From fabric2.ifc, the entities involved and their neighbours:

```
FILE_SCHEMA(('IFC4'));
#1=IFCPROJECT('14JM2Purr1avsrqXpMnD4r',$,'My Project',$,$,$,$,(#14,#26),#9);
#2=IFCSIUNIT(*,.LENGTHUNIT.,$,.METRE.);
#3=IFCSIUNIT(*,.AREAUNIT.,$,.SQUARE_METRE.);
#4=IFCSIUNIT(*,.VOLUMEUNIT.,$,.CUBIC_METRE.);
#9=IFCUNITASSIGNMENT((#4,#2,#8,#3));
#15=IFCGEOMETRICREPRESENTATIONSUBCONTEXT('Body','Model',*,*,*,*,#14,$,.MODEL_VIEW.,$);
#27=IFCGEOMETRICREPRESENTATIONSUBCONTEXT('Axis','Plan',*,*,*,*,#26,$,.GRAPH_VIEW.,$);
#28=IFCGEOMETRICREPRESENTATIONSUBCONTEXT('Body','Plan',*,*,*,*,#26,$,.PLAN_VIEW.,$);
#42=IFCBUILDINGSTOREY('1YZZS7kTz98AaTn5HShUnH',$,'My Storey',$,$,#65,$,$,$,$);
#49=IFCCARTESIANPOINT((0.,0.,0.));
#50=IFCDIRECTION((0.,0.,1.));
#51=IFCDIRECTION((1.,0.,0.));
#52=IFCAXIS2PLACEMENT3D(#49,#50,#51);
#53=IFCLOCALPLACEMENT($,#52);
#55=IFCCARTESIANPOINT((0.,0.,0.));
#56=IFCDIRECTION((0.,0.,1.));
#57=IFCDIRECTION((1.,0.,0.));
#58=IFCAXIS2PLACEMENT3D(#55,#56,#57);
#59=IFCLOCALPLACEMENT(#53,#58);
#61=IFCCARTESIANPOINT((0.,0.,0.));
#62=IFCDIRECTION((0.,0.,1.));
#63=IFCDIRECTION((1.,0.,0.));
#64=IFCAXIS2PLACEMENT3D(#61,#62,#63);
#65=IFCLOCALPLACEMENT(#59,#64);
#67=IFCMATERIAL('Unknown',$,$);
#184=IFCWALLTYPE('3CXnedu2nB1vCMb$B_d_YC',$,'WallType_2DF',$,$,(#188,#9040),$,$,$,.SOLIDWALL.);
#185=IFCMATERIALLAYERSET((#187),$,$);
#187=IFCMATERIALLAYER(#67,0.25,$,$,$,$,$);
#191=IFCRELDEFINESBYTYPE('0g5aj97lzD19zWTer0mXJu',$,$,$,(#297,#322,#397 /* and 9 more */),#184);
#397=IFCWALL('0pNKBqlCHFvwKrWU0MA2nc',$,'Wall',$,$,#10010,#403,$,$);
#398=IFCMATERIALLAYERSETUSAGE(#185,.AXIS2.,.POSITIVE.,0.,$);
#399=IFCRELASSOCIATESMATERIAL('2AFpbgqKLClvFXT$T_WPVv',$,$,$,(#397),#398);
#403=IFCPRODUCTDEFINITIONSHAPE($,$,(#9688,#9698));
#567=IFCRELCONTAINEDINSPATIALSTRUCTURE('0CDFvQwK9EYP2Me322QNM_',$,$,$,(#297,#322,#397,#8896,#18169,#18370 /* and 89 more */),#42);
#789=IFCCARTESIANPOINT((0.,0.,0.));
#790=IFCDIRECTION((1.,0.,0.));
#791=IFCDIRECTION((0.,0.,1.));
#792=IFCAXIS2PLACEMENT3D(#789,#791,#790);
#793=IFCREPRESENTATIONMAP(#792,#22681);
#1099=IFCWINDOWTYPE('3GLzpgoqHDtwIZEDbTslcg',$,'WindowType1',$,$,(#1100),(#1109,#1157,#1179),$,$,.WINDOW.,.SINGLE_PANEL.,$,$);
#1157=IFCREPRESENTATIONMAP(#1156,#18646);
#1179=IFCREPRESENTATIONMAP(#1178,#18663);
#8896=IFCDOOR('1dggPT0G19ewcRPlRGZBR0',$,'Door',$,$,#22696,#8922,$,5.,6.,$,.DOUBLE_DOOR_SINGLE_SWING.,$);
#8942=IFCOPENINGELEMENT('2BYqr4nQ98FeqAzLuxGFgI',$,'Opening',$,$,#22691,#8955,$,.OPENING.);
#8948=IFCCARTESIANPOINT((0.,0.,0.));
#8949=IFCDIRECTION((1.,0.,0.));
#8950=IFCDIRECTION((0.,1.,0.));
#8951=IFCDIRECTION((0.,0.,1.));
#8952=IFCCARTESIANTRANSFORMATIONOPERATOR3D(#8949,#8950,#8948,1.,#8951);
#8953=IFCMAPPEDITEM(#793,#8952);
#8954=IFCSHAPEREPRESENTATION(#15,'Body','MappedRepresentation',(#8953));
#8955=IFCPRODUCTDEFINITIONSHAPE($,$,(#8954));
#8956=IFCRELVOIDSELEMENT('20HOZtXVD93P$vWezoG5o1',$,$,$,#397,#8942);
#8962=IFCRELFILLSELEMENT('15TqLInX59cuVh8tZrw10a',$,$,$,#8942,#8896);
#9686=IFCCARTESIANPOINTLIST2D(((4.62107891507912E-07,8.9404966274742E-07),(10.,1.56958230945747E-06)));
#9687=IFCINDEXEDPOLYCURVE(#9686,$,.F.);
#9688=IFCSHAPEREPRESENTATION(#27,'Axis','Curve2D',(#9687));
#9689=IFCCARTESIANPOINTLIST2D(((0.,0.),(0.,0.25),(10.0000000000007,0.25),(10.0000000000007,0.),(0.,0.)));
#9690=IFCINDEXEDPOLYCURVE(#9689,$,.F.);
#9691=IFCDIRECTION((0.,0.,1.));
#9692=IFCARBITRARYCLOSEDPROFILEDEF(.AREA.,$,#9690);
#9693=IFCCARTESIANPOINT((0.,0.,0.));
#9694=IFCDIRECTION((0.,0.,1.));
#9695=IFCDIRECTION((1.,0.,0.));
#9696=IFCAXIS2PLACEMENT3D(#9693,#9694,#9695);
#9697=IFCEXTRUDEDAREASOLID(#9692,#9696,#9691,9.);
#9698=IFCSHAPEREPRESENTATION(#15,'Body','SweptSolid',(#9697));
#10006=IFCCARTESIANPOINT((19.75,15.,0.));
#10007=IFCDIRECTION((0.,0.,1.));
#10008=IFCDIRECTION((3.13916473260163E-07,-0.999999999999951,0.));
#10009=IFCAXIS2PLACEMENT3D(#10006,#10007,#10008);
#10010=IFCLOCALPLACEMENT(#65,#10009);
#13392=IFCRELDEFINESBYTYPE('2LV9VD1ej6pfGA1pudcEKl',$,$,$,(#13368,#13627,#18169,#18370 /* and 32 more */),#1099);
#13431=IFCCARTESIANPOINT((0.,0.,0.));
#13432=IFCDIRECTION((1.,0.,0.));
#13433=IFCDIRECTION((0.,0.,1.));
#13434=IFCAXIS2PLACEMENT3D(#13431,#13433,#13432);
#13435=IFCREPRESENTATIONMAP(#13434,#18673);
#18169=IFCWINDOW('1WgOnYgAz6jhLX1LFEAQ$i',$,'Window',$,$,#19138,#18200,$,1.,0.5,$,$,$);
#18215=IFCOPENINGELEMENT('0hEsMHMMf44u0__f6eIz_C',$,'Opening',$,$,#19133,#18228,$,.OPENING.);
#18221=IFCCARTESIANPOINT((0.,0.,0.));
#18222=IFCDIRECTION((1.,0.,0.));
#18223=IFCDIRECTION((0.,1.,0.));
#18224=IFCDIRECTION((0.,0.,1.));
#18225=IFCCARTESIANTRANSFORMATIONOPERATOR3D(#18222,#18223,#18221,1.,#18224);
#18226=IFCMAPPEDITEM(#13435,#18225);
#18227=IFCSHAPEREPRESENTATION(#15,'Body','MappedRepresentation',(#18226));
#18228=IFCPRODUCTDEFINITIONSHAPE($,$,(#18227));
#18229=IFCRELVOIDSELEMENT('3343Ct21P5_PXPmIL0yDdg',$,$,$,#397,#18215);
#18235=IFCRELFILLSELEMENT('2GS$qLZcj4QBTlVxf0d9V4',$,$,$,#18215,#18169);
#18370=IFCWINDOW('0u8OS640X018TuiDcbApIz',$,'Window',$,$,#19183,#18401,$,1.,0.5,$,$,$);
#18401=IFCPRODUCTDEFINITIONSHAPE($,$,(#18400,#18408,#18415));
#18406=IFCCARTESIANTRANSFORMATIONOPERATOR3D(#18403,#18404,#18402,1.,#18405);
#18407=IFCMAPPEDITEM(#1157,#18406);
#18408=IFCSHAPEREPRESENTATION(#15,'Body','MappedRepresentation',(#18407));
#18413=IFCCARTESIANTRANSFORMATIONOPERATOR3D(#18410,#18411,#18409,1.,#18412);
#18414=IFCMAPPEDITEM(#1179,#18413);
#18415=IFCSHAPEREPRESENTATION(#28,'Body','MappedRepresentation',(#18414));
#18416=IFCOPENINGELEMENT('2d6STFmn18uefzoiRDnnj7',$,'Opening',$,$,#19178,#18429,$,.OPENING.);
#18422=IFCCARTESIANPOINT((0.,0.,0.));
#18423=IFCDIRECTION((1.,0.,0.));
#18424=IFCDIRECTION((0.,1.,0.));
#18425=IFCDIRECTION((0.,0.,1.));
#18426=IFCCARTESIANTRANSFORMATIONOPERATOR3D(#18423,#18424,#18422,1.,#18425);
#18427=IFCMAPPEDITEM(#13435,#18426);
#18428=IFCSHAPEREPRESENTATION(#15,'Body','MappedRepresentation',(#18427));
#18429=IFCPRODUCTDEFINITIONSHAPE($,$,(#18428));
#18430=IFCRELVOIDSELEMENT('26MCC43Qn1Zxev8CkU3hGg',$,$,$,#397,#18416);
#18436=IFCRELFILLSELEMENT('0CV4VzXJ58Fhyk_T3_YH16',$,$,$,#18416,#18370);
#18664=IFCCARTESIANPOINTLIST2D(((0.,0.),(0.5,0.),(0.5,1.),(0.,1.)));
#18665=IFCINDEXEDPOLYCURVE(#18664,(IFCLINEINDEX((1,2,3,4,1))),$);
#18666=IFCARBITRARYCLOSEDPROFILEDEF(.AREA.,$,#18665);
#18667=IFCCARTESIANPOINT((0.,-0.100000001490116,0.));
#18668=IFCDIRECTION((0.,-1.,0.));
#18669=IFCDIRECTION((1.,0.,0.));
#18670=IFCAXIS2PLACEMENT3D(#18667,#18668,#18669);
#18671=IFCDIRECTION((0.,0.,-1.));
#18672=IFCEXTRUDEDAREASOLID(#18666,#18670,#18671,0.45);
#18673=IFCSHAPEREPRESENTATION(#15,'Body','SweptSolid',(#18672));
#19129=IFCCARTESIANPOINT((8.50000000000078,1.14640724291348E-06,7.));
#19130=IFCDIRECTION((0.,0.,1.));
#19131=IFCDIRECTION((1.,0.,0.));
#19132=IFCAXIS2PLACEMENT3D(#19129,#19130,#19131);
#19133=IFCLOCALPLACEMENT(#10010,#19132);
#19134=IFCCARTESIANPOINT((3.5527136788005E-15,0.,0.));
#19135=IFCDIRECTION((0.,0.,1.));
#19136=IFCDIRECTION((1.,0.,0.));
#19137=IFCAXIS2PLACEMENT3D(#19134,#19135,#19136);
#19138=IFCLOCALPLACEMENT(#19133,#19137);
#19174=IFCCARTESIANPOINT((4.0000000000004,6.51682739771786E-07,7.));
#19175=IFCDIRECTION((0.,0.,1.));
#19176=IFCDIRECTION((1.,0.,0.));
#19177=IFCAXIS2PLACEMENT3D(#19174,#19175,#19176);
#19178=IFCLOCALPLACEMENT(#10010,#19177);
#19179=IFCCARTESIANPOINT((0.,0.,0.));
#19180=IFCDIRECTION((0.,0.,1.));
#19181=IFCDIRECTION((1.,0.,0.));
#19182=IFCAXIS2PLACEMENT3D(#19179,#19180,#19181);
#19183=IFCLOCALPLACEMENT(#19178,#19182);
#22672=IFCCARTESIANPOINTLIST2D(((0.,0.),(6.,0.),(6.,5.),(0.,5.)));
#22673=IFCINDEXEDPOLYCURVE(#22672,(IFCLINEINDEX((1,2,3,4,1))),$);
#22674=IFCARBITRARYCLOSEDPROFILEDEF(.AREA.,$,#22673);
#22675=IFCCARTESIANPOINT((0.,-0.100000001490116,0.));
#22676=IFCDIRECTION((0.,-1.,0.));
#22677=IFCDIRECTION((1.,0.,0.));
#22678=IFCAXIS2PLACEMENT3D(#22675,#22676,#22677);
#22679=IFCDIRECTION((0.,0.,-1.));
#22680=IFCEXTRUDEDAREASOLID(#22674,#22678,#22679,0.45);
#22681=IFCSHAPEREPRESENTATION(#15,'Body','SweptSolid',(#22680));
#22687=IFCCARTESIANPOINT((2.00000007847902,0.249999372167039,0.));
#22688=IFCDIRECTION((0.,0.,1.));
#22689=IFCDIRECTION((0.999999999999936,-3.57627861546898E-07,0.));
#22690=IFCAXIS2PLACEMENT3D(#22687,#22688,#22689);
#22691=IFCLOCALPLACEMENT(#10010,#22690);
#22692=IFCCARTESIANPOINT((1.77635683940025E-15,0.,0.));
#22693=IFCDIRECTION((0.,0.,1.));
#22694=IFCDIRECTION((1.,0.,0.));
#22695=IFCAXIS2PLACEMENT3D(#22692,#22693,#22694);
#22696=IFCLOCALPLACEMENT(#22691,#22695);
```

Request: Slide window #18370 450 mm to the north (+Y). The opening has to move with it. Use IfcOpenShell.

```python
import ifcopenshell
import ifcopenshell.api.geometry
import ifcopenshell.util.placement
import ifcopenshell.util.unit

model = ifcopenshell.open("fabric2.ifc")
unit_scale = ifcopenshell.util.unit.calculate_unit_scale(model)

window = model.by_guid("0u8OS640X018TuiDcbApIz")
opening = window.FillsVoids[0].RelatingOpeningElement
wall = opening.VoidsElements[0].RelatingBuildingElement

wall_matrix = ifcopenshell.util.placement.get_local_placement(wall.ObjectPlacement)
shift = wall_matrix[:3, 0] * -0.45 / unit_scale
before = ifcopenshell.util.placement.get_local_placement(window.ObjectPlacement)[:3, 3].copy()

# The window is placed relative to its opening, so it follows when the opening moves.
matrix = ifcopenshell.util.placement.get_local_placement(opening.ObjectPlacement)
matrix[:3, 3] += shift
ifcopenshell.api.geometry.edit_object_placement(
    model, product=opening, matrix=matrix, is_si=False, should_transform_children=True
)

after = ifcopenshell.util.placement.get_local_placement(window.ObjectPlacement)[:3, 3]
print("window moved by", (after - before).round(3) + 0.0)

model.write("fabric2-out.ifc")
```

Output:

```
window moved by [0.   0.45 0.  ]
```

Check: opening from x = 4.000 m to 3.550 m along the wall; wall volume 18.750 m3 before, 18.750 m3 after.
